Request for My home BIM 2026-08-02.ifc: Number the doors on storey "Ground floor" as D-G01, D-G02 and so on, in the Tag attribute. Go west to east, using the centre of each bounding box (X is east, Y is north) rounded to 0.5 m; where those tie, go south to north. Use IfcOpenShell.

First a look at what the model holds.

```python
import ifcopenshell
import ifcopenshell.util.element
import ifcopenshell.util.placement

model = ifcopenshell.open("My home BIM 2026-08-02.ifc")
print(model.schema)
storey = next(s for s in model.by_type("IfcBuildingStorey") if s.Name == "Ground floor")
doors = [e for e in ifcopenshell.util.element.get_decomposition(storey) if e.is_a("IfcDoor")]
for e in sorted(doors, key=lambda e: e.id()):
    origin = ifcopenshell.util.placement.get_local_placement(e.ObjectPlacement)[:3, 3]
    print(e.id(), e.Tag, e.Name, origin.round(2) + 0.0, sep=" | ")
```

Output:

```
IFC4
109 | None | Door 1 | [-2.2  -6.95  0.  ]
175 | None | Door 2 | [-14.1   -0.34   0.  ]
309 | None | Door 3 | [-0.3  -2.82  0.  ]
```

```python
import ifcopenshell
import ifcopenshell.geom
import ifcopenshell.util.element
import ifcopenshell.util.shape

model = ifcopenshell.open("My home BIM 2026-08-02.ifc")
settings = ifcopenshell.geom.settings()
settings.set("use-world-coords", True)


def centre(element):
    shape = ifcopenshell.geom.create_shape(settings, element)
    return ifcopenshell.util.shape.get_bbox_centroid(shape.geometry)


storey = next(s for s in model.by_type("IfcBuildingStorey") if s.Name == "Ground floor")
doors = [e for e in ifcopenshell.util.element.get_decomposition(storey) if e.is_a("IfcDoor")]

# Insertion points can sit at a corner or the storey origin, so sort by the geometry (in metres).
centres = {e: centre(e) for e in doors}
doors.sort(key=lambda e: (round(centres[e][0] / 0.5), centres[e][1]))

for i, e in enumerate(doors, start=1):
    number = f"D-G{i:02d}"
    e.Tag = number
    print(e.id(), number)

model.write("My home BIM 2026-08-02-out.ifc")
```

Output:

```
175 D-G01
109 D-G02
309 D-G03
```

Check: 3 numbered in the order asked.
